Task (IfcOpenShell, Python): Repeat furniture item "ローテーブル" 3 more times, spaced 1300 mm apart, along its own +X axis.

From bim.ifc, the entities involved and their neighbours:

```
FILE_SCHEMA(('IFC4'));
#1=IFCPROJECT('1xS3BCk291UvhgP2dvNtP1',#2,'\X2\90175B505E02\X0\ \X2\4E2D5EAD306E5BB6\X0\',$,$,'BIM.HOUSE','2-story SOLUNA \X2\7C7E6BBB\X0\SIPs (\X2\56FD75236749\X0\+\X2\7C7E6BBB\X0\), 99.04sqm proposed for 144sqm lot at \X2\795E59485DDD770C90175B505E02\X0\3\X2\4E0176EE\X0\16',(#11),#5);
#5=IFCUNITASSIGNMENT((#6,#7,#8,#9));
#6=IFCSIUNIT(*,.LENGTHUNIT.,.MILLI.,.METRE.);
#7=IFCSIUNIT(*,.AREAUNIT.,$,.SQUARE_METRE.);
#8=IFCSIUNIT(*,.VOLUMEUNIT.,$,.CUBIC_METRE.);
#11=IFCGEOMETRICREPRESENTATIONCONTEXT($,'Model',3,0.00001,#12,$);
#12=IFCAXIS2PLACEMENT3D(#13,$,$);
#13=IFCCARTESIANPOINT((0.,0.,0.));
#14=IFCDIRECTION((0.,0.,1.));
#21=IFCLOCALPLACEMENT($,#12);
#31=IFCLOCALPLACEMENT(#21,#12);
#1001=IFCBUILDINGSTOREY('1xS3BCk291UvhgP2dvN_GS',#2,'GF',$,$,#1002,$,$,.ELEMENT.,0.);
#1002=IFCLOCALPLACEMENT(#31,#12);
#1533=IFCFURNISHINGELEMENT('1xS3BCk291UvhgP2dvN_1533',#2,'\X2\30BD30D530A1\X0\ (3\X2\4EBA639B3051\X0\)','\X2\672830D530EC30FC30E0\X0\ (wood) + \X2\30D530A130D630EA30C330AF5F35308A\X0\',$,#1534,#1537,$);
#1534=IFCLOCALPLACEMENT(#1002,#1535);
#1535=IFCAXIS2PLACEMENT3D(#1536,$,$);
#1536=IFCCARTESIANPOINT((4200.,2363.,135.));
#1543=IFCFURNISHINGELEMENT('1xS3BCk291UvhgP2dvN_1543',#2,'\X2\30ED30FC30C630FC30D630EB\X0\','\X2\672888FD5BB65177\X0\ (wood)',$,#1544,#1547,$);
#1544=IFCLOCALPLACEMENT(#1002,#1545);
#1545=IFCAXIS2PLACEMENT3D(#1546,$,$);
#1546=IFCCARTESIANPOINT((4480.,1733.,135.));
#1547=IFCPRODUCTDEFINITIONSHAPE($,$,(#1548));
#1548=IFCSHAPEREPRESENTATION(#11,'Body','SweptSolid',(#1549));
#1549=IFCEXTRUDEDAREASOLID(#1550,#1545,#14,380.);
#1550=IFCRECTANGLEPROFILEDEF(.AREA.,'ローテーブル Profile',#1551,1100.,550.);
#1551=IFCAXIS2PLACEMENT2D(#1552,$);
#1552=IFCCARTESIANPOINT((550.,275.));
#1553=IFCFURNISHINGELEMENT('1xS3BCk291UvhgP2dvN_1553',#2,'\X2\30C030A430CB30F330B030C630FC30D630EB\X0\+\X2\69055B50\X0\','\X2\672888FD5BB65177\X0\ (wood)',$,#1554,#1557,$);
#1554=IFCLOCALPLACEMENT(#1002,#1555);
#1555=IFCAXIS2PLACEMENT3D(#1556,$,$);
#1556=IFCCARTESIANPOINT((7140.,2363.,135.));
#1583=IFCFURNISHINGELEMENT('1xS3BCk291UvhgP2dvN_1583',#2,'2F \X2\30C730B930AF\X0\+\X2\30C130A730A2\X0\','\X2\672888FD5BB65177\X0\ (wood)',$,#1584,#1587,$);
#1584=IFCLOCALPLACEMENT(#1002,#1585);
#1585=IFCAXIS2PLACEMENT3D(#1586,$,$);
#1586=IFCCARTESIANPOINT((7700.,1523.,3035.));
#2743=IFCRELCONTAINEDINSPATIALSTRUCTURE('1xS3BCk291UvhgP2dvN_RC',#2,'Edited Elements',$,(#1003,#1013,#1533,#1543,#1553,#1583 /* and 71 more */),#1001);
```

```python
import ifcopenshell
import ifcopenshell.api.geometry
import ifcopenshell.api.root
import ifcopenshell.util.element
import ifcopenshell.util.placement
import ifcopenshell.util.unit

model = ifcopenshell.open("bim.ifc")
unit_scale = ifcopenshell.util.unit.calculate_unit_scale(model)


def reuse_history(source, copy):
    """copy_class also copies each property set's owner history, people and application; keep the originals."""
    for rel in copy.IsDefinedBy:
        if rel.is_a("IfcRelDefinesByProperties") and (history := rel.RelatingPropertyDefinition.OwnerHistory):
            rel.RelatingPropertyDefinition.OwnerHistory = source.OwnerHistory
            ifcopenshell.util.element.remove_deep2(model, history)


source = model.by_guid("1xS3BCk291UvhgP2dvN_1543")
base = ifcopenshell.util.placement.get_local_placement(source.ObjectPlacement)
step = base[:3, 0] * 1.3 / unit_scale

for i in range(1, 4):
    copy = ifcopenshell.api.root.copy_class(model, product=source)
    copy.Representation = ifcopenshell.util.element.copy_deep(
        model, source.Representation, exclude=["IfcGeometricRepresentationContext", "IfcRepresentationMap"]
    )
    reuse_history(source, copy)
    matrix = base.copy()
    matrix[:3, 3] += i * step
    print("added at", matrix[:3, 3].round(3) + 0.0)
    ifcopenshell.api.geometry.edit_object_placement(model, product=copy, matrix=matrix, is_si=False)

model.write("bim_v2.ifc")
```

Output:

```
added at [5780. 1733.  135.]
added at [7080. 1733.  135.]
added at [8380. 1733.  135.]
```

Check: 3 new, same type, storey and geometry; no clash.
